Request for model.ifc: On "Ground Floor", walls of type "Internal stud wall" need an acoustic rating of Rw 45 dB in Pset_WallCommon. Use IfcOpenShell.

First a look at what the model holds.

```python
import ifcopenshell
import ifcopenshell.util.element

model = ifcopenshell.open("model.ifc")
print(model.schema)
storey = next(s for s in model.by_type("IfcBuildingStorey") if s.Name == "Ground Floor")
walls = [e for e in ifcopenshell.util.element.get_decomposition(storey) if e.is_a("IfcWall")]
seen = {}
for e in walls:
    element_type = ifcopenshell.util.element.get_type(e)
    key = (element_type.Name if element_type != e and element_type else None, ifcopenshell.util.element.get_pset(e, "Pset_WallCommon", "AcousticRating"))
    seen[key] = seen.get(key, 0) + 1
for (name, value), count in sorted(seen.items(), key=str):
    print(count, "x", name, "|", value)
```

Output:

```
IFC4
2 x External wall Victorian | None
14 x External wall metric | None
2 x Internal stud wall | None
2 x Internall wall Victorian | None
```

```python
import ifcopenshell
import ifcopenshell.api.pset
import ifcopenshell.util.element

model = ifcopenshell.open("model.ifc")

storey = next(s for s in model.by_type("IfcBuildingStorey") if s.Name == "Ground Floor")
walls = [e for e in ifcopenshell.util.element.get_decomposition(storey) if e.is_a("IfcWall")]

count = 0
for e in walls:
    element_type = ifcopenshell.util.element.get_type(e)
    if element_type in (None, e) or element_type.Name != "Internal stud wall":
        continue
    # add_pset returns the element's existing set when there is one.
    pset = ifcopenshell.api.pset.add_pset(model, product=e, name="Pset_WallCommon")
    ifcopenshell.api.pset.edit_pset(model, pset=pset, properties={"AcousticRating": "Rw 45 dB"})
    count += 1

print(count, "walls updated")

model.write("model_updated.ifc")
```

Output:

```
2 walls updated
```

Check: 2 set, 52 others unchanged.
